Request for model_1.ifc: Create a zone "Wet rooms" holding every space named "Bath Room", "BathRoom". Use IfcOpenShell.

First a look at what the model holds.

```python
import ifcopenshell

model = ifcopenshell.open("model_1.ifc")
print(model.schema)
seen = {}
for space in model.by_type("IfcSpace"):
    seen[space.LongName] = seen.get(space.LongName, 0) + 1
for name, count in sorted(seen.items(), key=str):
    print(count, "x", name)
print("zones:", [z.Name for z in model.by_type("IfcZone")][:20])
```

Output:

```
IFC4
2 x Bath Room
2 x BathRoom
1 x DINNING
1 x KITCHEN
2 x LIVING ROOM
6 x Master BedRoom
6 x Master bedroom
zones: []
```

```python
import ifcopenshell
import ifcopenshell.api.group
import ifcopenshell.api.root

model = ifcopenshell.open("model_1.ifc")

names = {"Bath Room", "BathRoom"}
spaces = [s for s in model.by_type("IfcSpace") if s.LongName in names]

zone = ifcopenshell.api.root.create_entity(model, ifc_class="IfcZone", name="Wet rooms")
ifcopenshell.api.group.assign_group(model, products=spaces, group=zone)
print(len(spaces), "spaces in", zone.Name)

model.write("model_1_v2.ifc")
```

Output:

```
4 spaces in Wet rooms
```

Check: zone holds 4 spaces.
